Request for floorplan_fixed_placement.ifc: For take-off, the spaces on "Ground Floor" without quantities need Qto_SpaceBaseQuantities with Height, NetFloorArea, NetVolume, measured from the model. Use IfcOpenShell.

First a look at what the model holds.

```python
import ifcopenshell
import ifcopenshell.util.element
import ifcopenshell.util.unit

model = ifcopenshell.open("floorplan_fixed_placement.ifc")
print(model.schema)
for unit_type in ("LENGTHUNIT", "AREAUNIT", "VOLUMEUNIT"):
    print(unit_type, ifcopenshell.util.unit.calculate_unit_scale(model, unit_type))
storey = next(s for s in model.by_type("IfcBuildingStorey") if s.Name == "Ground Floor")
spaces = [e for e in ifcopenshell.util.element.get_decomposition(storey) if e.is_a("IfcSpace")]
for e in sorted(spaces, key=lambda e: e.id()):
    print(e.id(), e.is_a(), e.Name, list(ifcopenshell.util.element.get_psets(e, qtos_only=True)), sep=" | ")
```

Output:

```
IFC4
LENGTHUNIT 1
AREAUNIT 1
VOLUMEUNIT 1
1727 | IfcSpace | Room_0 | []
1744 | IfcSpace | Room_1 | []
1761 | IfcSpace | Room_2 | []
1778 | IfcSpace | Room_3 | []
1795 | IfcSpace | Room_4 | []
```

```python
import ifcopenshell
import ifcopenshell.api.pset
import ifcopenshell.geom
import ifcopenshell.util.element
import ifcopenshell.util.shape
import ifcopenshell.util.unit

model = ifcopenshell.open("floorplan_fixed_placement.ifc")
unit_scale = ifcopenshell.util.unit.calculate_unit_scale(model)
area_scale = ifcopenshell.util.unit.calculate_unit_scale(model, "AREAUNIT")
volume_scale = ifcopenshell.util.unit.calculate_unit_scale(model, "VOLUMEUNIT")
settings = ifcopenshell.geom.settings()

storey = next(s for s in model.by_type("IfcBuildingStorey") if s.Name == "Ground Floor")
spaces = [e for e in ifcopenshell.util.element.get_decomposition(storey) if e.is_a("IfcSpace")]

for e in sorted(spaces, key=lambda e: e.id()):
    if ifcopenshell.util.element.get_psets(e, qtos_only=True, should_inherit=False):
        continue
    # Geometry comes back in metres, in the element's own axes.
    shape = ifcopenshell.geom.create_shape(settings, e)
    values = {
        "Height": ifcopenshell.util.shape.get_z(shape.geometry) / unit_scale,
        "NetFloorArea": ifcopenshell.util.shape.get_footprint_area(shape.geometry) / area_scale,
        "NetVolume": ifcopenshell.util.shape.get_volume(shape.geometry) / volume_scale,
    }
    qto = ifcopenshell.api.pset.add_qto(model, product=e, name="Qto_SpaceBaseQuantities")
    ifcopenshell.api.pset.edit_qto(model, qto=qto, properties=values)
    print(e.id(), {k: round(v, 3) for k, v in values.items()})

model.write("floorplan_fixed_placement_v2.ifc")
```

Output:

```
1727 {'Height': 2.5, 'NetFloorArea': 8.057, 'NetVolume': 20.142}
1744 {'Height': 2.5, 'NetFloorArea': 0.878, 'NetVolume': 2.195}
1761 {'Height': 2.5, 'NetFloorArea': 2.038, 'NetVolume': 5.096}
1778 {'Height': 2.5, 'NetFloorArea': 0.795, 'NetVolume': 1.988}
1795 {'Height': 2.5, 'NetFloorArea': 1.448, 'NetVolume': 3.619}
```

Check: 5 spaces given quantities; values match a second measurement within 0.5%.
